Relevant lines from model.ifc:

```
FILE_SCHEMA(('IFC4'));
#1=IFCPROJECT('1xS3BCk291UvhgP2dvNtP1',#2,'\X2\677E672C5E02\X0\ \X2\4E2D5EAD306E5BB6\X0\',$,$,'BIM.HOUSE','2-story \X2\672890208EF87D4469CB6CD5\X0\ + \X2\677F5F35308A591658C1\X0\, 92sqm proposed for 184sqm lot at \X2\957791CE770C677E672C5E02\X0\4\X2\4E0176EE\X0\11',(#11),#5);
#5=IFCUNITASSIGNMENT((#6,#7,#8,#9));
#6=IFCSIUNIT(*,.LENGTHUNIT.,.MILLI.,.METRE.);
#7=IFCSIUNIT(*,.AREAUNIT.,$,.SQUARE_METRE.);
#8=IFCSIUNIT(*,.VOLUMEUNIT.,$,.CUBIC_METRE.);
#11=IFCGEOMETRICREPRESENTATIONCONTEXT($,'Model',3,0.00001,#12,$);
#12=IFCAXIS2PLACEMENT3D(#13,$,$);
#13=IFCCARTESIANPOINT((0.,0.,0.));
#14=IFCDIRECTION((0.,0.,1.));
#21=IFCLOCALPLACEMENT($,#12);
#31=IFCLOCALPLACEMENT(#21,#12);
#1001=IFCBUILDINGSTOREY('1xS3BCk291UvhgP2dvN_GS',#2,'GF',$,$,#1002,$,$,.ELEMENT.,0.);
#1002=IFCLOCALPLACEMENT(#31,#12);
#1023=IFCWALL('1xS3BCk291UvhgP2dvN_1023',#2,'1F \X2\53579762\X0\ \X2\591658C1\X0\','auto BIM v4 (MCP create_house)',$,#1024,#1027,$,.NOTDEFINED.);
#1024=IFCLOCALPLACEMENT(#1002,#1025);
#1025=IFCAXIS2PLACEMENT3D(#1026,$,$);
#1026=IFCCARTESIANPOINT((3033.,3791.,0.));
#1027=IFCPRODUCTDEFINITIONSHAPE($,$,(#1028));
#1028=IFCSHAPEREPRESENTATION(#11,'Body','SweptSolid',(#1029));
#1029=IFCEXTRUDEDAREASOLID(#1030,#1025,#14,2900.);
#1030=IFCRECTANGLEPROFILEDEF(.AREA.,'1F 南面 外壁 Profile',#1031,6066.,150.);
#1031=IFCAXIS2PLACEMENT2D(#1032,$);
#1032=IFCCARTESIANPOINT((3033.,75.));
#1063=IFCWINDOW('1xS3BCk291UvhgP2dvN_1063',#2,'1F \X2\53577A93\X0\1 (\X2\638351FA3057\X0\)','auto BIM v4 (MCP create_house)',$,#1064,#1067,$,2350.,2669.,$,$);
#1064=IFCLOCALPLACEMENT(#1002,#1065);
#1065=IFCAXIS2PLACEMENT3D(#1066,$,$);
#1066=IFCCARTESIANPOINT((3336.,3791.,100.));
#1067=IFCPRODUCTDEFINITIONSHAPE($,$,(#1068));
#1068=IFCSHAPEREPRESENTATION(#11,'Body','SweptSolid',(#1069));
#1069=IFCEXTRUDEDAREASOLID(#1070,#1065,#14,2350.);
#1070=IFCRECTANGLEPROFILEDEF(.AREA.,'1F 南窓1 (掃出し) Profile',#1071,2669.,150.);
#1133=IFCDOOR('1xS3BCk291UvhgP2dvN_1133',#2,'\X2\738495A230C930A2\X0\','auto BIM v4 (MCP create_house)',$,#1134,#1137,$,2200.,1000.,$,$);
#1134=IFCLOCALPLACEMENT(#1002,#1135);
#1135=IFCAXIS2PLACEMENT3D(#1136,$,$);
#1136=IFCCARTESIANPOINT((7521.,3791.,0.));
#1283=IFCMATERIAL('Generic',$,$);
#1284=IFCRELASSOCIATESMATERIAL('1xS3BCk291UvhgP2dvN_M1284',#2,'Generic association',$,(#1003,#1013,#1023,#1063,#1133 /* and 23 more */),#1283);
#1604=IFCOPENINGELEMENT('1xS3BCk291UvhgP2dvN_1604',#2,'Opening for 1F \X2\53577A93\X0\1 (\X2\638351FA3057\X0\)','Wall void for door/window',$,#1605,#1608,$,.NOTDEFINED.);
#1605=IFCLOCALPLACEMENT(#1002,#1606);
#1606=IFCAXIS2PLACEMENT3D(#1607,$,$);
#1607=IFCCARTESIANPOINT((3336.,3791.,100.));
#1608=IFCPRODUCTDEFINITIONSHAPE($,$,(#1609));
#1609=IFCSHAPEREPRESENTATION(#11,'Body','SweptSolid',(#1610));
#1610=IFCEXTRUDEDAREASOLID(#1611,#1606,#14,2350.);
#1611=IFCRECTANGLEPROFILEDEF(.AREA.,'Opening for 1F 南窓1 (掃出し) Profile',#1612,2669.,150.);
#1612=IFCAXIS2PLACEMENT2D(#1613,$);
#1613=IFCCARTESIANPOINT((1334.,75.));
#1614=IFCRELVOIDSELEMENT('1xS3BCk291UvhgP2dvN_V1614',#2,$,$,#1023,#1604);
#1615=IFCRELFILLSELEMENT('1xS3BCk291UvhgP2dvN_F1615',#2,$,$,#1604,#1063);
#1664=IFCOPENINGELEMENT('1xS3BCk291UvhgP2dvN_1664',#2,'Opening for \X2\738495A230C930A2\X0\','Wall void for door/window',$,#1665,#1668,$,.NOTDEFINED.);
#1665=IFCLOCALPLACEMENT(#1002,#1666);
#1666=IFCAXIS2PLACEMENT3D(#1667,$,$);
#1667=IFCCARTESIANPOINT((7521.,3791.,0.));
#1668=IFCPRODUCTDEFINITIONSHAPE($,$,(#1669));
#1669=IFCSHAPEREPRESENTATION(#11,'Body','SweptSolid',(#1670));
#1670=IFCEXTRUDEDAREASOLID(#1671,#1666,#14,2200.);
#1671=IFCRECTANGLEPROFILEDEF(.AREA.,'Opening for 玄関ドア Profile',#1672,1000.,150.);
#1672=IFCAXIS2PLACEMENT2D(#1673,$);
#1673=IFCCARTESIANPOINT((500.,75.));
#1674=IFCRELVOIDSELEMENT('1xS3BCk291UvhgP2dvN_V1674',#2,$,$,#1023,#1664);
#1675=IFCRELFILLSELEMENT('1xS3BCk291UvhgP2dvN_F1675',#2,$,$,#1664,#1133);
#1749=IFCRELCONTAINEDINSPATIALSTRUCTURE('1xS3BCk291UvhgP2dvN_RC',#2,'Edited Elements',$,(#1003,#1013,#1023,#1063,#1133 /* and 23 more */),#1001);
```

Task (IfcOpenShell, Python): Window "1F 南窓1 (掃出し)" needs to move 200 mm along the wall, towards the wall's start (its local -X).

```python
import ifcopenshell
import ifcopenshell.api.geometry
import ifcopenshell.util.placement

model = ifcopenshell.open("model.ifc")

window = model.by_id(1063)
opening = window.FillsVoids[0].RelatingOpeningElement
wall = opening.VoidsElements[0].RelatingBuildingElement

wall_matrix = ifcopenshell.util.placement.get_local_placement(wall.ObjectPlacement)
shift = wall_matrix[:3, 0] * -200.0
before = ifcopenshell.util.placement.get_local_placement(window.ObjectPlacement)[:3, 3].copy()

# The window is not placed relative to its opening, so move both.
for product in (opening, window):
    matrix = ifcopenshell.util.placement.get_local_placement(product.ObjectPlacement)
    matrix[:3, 3] += shift
    ifcopenshell.api.geometry.edit_object_placement(model, product=product, matrix=matrix, is_si=False)

after = ifcopenshell.util.placement.get_local_placement(window.ObjectPlacement)[:3, 3]
print("window moved by", (after - before).round(3) + 0.0)

model.write("model_rev.ifc")
```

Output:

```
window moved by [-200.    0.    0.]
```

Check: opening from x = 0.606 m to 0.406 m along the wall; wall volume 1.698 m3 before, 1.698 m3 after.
